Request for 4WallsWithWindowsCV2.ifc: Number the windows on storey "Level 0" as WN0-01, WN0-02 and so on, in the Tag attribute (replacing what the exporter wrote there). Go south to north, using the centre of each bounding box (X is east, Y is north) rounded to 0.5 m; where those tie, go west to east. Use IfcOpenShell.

First a look at what the model holds.

```python
import ifcopenshell
import ifcopenshell.util.element
import ifcopenshell.util.placement

model = ifcopenshell.open("4WallsWithWindowsCV2.ifc")
print(model.schema)
storey = next(s for s in model.by_type("IfcBuildingStorey") if s.Name == "Level 0")
windows = [e for e in ifcopenshell.util.element.get_decomposition(storey) if e.is_a("IfcWindow")]
for e in sorted(windows, key=lambda e: e.id()):
    origin = ifcopenshell.util.placement.get_local_placement(e.ObjectPlacement)[:3, 3]
    print(e.id(), e.Tag, e.Name, origin.round(2) + 0.0, sep=" | ")
```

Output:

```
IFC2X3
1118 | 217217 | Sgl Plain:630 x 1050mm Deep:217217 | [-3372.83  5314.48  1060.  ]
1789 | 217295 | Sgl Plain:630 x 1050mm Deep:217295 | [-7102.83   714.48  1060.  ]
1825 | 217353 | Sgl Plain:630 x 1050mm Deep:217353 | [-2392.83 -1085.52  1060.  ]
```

```python
import ifcopenshell
import ifcopenshell.geom
import ifcopenshell.util.element
import ifcopenshell.util.shape

model = ifcopenshell.open("4WallsWithWindowsCV2.ifc")
settings = ifcopenshell.geom.settings()
settings.set("use-world-coords", True)


def centre(element):
    shape = ifcopenshell.geom.create_shape(settings, element)
    return ifcopenshell.util.shape.get_bbox_centroid(shape.geometry)


storey = next(s for s in model.by_type("IfcBuildingStorey") if s.Name == "Level 0")
windows = [e for e in ifcopenshell.util.element.get_decomposition(storey) if e.is_a("IfcWindow")]

# Insertion points can sit at a corner or the storey origin, so sort by the geometry (in metres).
centres = {e: centre(e) for e in windows}
windows.sort(key=lambda e: (round(centres[e][1] / 0.5), centres[e][0]))

for i, e in enumerate(windows, start=1):
    number = f"WN0-{i:02d}"
    e.Tag = number
    print(e.id(), number)

model.write("4WallsWithWindowsCV2_edited.ifc")
```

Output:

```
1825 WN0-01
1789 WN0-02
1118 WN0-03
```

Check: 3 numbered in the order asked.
